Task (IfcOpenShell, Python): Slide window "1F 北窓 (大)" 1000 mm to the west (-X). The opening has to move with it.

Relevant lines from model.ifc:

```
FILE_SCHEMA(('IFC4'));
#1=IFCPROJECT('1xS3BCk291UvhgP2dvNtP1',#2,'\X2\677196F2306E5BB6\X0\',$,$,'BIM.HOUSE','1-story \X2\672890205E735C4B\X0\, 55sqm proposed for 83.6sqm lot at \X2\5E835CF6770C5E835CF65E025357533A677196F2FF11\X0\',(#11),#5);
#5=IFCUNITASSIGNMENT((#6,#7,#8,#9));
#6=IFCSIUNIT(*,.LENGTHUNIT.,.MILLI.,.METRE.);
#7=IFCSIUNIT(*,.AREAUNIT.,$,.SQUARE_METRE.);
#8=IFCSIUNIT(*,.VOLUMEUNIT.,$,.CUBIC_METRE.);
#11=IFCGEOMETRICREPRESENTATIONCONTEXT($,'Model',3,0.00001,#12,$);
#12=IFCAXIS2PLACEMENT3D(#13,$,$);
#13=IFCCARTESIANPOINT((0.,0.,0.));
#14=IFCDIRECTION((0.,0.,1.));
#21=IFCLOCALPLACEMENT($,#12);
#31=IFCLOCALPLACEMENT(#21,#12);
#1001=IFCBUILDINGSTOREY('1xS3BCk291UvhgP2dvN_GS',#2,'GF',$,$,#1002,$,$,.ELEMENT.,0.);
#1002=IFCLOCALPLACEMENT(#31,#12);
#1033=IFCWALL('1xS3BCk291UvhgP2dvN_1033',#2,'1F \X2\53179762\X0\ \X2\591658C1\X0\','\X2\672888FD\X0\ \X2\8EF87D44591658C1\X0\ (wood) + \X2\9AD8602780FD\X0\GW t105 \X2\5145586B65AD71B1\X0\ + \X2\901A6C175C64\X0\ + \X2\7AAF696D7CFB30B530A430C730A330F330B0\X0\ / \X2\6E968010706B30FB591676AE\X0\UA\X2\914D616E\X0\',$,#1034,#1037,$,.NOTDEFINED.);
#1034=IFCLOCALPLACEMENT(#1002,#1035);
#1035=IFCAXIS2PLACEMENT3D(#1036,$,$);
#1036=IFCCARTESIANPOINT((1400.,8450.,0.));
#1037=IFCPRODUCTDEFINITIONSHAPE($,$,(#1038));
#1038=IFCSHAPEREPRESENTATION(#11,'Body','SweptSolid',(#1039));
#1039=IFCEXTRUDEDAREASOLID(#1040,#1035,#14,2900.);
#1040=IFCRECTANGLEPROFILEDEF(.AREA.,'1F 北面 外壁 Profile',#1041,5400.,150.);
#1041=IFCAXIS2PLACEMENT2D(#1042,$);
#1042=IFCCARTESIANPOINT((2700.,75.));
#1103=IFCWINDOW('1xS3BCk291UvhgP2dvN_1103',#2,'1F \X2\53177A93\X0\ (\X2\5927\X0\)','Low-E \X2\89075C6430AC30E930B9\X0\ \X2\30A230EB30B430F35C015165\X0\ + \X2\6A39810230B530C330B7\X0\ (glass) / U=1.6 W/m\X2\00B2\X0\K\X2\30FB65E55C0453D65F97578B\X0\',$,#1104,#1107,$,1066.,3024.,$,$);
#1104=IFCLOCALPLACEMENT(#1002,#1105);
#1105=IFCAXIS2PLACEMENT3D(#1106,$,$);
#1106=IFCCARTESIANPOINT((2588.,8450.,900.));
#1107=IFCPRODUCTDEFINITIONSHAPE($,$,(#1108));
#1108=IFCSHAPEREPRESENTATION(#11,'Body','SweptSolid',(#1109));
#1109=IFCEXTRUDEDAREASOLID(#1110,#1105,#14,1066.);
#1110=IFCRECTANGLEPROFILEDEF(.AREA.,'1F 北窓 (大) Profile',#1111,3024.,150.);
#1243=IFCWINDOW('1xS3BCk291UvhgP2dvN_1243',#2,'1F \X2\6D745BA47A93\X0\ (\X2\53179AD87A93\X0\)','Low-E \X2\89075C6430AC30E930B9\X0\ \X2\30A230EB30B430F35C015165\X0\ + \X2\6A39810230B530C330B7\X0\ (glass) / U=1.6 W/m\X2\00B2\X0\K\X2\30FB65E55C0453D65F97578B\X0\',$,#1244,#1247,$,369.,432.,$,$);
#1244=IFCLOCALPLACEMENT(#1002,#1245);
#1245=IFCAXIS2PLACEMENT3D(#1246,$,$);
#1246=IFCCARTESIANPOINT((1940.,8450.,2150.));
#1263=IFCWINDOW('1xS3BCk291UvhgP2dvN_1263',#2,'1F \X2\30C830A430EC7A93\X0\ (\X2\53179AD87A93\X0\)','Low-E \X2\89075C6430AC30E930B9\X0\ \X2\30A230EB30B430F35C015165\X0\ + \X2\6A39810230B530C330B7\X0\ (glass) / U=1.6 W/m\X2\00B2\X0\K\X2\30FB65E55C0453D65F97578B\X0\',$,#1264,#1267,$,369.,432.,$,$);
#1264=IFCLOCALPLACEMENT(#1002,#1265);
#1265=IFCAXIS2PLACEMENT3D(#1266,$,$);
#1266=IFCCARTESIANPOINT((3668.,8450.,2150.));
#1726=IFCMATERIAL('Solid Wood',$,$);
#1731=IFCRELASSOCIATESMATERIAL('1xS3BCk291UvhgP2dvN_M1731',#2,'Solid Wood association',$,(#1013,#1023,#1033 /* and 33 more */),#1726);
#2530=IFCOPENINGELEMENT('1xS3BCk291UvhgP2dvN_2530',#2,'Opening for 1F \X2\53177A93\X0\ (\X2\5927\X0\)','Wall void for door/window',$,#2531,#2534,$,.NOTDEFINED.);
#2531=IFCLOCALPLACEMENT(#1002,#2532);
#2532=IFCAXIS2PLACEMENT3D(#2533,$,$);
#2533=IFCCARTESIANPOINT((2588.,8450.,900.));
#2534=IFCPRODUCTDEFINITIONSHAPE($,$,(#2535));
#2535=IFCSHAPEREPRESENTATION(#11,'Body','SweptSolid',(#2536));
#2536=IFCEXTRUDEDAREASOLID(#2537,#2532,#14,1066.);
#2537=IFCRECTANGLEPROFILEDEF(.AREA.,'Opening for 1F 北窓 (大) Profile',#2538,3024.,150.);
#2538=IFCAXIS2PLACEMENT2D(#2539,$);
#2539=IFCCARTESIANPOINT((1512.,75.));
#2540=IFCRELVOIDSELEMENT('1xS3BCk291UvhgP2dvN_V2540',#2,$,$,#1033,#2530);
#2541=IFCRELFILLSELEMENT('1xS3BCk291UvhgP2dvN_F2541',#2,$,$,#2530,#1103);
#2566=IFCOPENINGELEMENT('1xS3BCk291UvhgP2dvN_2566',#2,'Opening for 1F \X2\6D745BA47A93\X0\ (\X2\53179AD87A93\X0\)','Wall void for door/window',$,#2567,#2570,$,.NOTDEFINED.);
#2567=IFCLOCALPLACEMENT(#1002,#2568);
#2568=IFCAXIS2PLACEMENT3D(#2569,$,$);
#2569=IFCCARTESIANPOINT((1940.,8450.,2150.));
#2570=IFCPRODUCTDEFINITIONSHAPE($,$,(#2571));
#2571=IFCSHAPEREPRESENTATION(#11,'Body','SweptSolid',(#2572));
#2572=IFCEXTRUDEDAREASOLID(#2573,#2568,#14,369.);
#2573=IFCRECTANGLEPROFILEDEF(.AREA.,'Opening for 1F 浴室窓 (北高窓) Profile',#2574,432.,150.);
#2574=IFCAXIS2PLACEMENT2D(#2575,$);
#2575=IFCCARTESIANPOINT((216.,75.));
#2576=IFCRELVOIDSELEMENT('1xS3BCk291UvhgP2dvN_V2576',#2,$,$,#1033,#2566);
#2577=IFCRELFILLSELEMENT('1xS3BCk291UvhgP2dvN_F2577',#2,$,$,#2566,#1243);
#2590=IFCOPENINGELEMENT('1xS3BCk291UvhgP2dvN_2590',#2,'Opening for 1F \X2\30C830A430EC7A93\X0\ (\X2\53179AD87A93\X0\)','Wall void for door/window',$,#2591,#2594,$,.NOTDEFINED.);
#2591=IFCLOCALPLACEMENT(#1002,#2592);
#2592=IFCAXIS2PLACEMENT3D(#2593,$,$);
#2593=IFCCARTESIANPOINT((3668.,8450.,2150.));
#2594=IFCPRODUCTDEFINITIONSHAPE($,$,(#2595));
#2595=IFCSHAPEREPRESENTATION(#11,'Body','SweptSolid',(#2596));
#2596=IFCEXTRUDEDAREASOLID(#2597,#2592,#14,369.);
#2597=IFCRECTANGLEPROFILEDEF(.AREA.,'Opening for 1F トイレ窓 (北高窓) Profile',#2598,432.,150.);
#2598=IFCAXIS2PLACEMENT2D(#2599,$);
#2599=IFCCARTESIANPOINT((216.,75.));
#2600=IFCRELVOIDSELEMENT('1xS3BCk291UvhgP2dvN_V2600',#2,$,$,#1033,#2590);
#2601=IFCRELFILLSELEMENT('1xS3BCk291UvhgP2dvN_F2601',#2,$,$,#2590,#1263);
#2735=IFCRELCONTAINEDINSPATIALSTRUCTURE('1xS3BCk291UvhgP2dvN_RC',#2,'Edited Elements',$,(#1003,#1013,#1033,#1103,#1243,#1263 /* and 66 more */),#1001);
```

```python
import ifcopenshell
import ifcopenshell.api.geometry
import ifcopenshell.util.placement
import ifcopenshell.util.unit

model = ifcopenshell.open("model.ifc")
unit_scale = ifcopenshell.util.unit.calculate_unit_scale(model)

window = model.by_guid("1xS3BCk291UvhgP2dvN_1103")
opening = window.FillsVoids[0].RelatingOpeningElement
wall = opening.VoidsElements[0].RelatingBuildingElement

wall_matrix = ifcopenshell.util.placement.get_local_placement(wall.ObjectPlacement)
shift = wall_matrix[:3, 0] * -1 / unit_scale
before = ifcopenshell.util.placement.get_local_placement(window.ObjectPlacement)[:3, 3].copy()

# The window is not placed relative to its opening, so move both.
for product in (opening, window):
    matrix = ifcopenshell.util.placement.get_local_placement(product.ObjectPlacement)
    matrix[:3, 3] += shift
    ifcopenshell.api.geometry.edit_object_placement(model, product=product, matrix=matrix, is_si=False)

after = ifcopenshell.util.placement.get_local_placement(window.ObjectPlacement)[:3, 3]
print("window moved by", (after - before).round(3) + 0.0)

model.write("model_edited.ifc")
```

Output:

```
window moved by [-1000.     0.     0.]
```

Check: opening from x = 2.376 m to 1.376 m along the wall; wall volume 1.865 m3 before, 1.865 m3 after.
